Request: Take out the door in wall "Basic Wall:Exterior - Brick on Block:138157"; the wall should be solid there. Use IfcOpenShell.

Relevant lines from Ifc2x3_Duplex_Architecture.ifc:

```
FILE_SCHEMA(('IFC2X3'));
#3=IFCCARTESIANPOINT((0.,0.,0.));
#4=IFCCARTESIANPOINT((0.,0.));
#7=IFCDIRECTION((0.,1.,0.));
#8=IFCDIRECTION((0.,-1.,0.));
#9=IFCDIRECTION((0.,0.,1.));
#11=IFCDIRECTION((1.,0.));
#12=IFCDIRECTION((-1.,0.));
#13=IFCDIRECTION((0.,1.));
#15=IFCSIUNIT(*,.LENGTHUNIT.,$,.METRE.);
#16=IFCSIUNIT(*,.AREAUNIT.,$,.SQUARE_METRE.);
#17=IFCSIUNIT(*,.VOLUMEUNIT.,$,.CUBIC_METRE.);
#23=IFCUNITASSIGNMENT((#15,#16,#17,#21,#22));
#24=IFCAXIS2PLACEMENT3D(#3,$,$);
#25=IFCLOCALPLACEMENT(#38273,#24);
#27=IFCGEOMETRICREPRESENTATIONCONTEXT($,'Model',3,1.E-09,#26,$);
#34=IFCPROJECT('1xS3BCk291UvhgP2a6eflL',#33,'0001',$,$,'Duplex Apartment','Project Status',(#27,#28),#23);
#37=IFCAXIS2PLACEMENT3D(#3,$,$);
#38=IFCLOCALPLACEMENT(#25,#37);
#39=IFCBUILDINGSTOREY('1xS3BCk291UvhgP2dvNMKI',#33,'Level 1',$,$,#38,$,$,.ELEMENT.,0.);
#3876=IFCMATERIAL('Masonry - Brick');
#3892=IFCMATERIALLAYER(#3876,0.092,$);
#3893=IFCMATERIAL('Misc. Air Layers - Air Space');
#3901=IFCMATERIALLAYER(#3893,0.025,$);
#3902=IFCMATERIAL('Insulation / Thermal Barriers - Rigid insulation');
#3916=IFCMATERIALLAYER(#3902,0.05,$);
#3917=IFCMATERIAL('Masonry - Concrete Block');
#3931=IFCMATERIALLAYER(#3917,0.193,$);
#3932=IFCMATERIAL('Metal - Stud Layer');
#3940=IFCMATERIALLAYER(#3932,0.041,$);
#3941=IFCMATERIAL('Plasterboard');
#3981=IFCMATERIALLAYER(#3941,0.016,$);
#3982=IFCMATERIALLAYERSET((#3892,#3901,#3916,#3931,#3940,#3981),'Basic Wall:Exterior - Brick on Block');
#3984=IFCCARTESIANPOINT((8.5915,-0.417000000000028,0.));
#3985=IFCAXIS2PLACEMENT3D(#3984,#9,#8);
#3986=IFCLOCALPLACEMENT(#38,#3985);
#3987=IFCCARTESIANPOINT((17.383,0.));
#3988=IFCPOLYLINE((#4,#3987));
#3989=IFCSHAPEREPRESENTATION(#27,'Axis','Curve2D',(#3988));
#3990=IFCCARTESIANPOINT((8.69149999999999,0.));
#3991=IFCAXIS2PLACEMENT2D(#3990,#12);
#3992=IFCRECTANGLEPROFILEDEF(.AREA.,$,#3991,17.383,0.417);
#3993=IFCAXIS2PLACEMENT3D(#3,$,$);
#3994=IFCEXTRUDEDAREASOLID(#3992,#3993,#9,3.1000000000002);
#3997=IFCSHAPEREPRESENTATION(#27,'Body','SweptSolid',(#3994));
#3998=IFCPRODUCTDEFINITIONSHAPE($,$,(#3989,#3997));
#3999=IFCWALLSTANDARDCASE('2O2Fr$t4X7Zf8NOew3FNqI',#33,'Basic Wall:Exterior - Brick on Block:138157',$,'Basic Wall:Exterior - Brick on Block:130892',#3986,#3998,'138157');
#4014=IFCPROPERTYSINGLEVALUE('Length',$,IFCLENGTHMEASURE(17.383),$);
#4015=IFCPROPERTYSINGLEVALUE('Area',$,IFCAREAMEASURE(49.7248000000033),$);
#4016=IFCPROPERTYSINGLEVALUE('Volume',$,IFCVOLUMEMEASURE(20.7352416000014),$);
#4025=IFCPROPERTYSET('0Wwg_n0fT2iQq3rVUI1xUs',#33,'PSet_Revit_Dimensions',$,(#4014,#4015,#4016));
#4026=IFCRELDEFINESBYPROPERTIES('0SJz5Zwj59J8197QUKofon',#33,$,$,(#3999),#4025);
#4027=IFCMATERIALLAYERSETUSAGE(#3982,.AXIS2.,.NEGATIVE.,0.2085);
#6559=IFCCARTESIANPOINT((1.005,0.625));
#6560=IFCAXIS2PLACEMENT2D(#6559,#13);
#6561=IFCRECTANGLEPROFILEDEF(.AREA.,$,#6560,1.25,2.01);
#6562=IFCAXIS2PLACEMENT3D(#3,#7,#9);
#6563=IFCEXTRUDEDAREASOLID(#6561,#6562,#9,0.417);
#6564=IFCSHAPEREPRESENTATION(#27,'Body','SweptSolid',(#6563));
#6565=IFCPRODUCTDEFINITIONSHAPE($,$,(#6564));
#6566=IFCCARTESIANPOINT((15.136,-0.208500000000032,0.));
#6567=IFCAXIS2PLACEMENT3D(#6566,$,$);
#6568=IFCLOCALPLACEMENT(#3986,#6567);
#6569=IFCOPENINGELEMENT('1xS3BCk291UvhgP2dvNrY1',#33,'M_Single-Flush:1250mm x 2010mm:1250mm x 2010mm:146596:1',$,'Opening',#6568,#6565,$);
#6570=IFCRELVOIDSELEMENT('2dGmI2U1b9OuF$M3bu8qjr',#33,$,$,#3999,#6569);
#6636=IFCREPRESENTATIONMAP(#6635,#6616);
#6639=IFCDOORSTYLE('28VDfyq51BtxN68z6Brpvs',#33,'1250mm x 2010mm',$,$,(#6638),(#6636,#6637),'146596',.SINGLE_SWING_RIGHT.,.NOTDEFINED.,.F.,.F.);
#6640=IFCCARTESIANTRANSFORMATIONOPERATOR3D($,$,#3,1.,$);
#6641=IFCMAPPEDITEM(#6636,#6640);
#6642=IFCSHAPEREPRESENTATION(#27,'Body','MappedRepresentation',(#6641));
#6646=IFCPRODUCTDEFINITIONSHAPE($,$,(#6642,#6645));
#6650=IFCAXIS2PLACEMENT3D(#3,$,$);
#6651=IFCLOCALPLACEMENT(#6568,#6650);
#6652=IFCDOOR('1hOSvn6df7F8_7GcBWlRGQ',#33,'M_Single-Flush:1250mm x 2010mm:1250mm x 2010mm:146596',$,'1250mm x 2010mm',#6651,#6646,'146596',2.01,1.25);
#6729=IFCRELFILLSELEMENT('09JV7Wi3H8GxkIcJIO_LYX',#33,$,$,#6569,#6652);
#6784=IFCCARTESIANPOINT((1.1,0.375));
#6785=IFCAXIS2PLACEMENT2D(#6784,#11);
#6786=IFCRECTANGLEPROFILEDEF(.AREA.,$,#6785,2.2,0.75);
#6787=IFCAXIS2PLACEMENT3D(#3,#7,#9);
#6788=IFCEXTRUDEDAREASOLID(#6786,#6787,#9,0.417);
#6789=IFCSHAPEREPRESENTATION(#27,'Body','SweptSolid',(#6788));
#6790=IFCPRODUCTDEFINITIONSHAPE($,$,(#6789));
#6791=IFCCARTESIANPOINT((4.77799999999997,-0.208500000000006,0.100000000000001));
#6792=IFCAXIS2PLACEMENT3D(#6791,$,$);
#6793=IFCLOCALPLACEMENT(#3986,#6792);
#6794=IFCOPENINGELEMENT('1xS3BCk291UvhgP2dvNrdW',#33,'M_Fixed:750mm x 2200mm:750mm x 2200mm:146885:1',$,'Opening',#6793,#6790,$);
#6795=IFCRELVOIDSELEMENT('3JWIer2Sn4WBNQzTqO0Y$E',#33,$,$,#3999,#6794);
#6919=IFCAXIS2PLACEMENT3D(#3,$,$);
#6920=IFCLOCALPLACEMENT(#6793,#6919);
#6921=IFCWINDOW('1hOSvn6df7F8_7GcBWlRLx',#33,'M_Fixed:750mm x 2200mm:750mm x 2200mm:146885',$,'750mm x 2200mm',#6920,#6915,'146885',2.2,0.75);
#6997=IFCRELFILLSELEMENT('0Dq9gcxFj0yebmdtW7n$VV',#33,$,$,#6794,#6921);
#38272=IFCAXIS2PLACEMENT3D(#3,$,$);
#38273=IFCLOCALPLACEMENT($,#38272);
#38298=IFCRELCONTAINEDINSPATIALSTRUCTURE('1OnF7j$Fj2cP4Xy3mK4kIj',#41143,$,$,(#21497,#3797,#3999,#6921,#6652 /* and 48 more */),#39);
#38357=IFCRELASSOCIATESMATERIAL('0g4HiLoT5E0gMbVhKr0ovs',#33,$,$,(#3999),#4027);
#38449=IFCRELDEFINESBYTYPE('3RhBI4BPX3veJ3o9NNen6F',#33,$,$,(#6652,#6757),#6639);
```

```python
import ifcopenshell
import ifcopenshell.api.feature
import ifcopenshell.api.pset
import ifcopenshell.api.root
import ifcopenshell.geom
import ifcopenshell.util.element
import ifcopenshell.util.shape
import ifcopenshell.util.unit

model = ifcopenshell.open("Ifc2x3_Duplex_Architecture.ifc")
area_scale = ifcopenshell.util.unit.calculate_unit_scale(model, "AREAUNIT")
volume_scale = ifcopenshell.util.unit.calculate_unit_scale(model, "VOLUMEUNIT")
settings = ifcopenshell.geom.settings()


def volume(element):
    """Net volume in cubic metres, openings subtracted."""
    shape = ifcopenshell.geom.create_shape(settings, element)
    return ifcopenshell.util.shape.get_volume(shape.geometry)


door = model.by_guid("1hOSvn6df7F8_7GcBWlRGQ")
opening = door.FillsVoids[0].RelatingOpeningElement
wall = opening.VoidsElements[0].RelatingBuildingElement
before = volume(wall)

ifcopenshell.api.root.remove_product(model, product=door)
ifcopenshell.api.feature.remove_feature(model, feature=opening)

after = volume(wall)
thickness = 0.417  # wall thickness in metres

# Update the wall's stored quantities.
pset = model.by_id(ifcopenshell.util.element.get_pset(wall, "PSet_Revit_Dimensions", should_inherit=False)["id"])
ifcopenshell.api.pset.edit_pset(model, pset=pset, properties={
    "Area": model.create_entity("IfcAreaMeasure", after / thickness / area_scale),
    "Volume": model.create_entity("IfcVolumeMeasure", after / volume_scale),
})

print(f"wall volume {before:.3f} -> {after:.3f} m3")

model.write("Ifc2x3_Duplex_Architecture_rev.ifc")
```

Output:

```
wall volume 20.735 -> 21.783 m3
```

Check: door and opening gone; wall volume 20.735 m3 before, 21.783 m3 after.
